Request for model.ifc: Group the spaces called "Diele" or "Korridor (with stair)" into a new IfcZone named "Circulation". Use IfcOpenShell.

First a look at what the model holds.

```python
import ifcopenshell

model = ifcopenshell.open("model.ifc")
print(model.schema)
seen = {}
for space in model.by_type("IfcSpace"):
    seen[space.LongName] = seen.get(space.LongName, 0) + 1
for name, count in sorted(seen.items(), key=str):
    print(count, "x", name)
print("zones:", [z.Name for z in model.by_type("IfcZone")][:20])
```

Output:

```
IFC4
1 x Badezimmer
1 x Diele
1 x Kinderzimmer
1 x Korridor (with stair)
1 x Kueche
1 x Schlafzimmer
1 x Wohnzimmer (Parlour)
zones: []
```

```python
import ifcopenshell
import ifcopenshell.api.group
import ifcopenshell.api.root

model = ifcopenshell.open("model.ifc")

names = {"Diele", "Korridor (with stair)"}
spaces = [s for s in model.by_type("IfcSpace") if s.LongName in names]

zone = ifcopenshell.api.root.create_entity(model, ifc_class="IfcZone", name="Circulation")
ifcopenshell.api.group.assign_group(model, products=spaces, group=zone)
print(len(spaces), "spaces in", zone.Name)

model.write("model_v2.ifc")
```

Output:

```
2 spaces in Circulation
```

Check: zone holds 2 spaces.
